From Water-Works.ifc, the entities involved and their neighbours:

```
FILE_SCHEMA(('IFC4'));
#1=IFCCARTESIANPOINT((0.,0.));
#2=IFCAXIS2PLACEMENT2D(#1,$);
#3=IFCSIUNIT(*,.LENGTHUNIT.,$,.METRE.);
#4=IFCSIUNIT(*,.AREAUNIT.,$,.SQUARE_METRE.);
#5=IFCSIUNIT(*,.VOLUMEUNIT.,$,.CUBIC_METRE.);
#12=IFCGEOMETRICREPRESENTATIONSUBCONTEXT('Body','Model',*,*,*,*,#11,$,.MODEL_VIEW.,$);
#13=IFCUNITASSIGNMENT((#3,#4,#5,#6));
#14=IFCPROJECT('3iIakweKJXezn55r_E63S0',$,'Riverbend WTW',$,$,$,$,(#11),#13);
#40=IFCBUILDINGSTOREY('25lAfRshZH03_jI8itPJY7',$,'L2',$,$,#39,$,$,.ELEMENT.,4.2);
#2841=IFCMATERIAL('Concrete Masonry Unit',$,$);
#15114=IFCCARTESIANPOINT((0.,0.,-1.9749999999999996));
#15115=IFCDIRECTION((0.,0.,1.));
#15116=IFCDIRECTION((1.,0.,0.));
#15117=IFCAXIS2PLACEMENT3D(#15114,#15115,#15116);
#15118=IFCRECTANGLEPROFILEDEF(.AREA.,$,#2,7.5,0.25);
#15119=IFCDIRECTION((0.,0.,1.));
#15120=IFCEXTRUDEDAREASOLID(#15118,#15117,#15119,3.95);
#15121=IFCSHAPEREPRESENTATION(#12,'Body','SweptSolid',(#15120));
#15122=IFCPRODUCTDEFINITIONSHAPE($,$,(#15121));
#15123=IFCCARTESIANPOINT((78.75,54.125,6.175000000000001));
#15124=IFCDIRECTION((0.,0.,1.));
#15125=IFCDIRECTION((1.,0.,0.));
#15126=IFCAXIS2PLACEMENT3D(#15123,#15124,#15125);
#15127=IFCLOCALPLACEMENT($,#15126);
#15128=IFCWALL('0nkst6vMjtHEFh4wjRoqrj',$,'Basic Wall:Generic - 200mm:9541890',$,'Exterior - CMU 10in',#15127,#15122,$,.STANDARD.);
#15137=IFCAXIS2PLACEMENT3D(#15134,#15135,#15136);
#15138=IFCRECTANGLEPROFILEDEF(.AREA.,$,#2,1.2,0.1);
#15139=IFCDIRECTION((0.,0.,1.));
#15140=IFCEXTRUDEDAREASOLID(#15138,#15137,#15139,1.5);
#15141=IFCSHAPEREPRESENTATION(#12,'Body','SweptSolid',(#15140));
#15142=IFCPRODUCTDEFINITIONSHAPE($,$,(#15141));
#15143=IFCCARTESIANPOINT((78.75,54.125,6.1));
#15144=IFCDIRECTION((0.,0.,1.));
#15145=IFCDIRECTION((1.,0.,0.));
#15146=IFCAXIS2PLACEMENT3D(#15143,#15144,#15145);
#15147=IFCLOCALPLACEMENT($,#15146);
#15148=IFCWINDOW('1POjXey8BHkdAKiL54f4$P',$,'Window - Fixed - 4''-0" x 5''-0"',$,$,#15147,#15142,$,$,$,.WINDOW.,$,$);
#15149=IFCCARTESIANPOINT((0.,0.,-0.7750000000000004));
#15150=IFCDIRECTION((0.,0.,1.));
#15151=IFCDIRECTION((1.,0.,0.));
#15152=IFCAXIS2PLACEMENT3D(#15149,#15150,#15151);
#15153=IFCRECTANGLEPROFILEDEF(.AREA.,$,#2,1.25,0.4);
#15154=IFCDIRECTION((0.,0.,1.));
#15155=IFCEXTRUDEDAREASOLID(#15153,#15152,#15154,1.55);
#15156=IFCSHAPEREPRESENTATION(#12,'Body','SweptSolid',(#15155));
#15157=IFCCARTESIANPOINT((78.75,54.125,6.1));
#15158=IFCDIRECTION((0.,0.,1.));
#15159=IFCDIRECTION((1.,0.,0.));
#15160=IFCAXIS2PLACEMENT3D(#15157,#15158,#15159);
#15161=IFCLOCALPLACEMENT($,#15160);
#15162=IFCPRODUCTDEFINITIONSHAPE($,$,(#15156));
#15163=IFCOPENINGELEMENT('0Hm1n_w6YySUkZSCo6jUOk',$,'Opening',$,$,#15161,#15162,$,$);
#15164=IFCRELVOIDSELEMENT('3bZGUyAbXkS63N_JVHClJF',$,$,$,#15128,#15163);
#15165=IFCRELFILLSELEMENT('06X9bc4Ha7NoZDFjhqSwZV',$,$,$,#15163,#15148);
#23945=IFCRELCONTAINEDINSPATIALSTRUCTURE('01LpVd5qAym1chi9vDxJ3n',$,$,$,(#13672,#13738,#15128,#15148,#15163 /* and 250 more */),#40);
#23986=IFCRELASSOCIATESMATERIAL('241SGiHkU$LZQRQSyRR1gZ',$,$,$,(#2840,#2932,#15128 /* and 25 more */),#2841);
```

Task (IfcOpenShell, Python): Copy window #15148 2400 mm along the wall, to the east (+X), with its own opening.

```python
import ifcopenshell
import ifcopenshell.api.feature
import ifcopenshell.api.geometry
import ifcopenshell.api.root
import ifcopenshell.geom
import ifcopenshell.util.element
import ifcopenshell.util.placement
import ifcopenshell.util.shape

model = ifcopenshell.open("Water-Works.ifc")
settings = ifcopenshell.geom.settings()


def volume(element):
    """Net volume in cubic metres, openings subtracted."""
    shape = ifcopenshell.geom.create_shape(settings, element)
    return ifcopenshell.util.shape.get_volume(shape.geometry)


window = model.by_guid("1POjXey8BHkdAKiL54f4$P")
opening = window.FillsVoids[0].RelatingOpeningElement
wall = opening.VoidsElements[0].RelatingBuildingElement
before = volume(wall)
shift = ifcopenshell.util.placement.get_local_placement(wall.ObjectPlacement)[:3, 0] * 2.4

# copy_class copies the void relationship, type, container and properties, but no geometry.
new_opening = ifcopenshell.api.root.copy_class(model, product=opening)
new_opening.Representation = ifcopenshell.util.element.copy_deep(
    model, opening.Representation, exclude=["IfcGeometricRepresentationContext", "IfcRepresentationMap"]
)
new_window = ifcopenshell.api.root.copy_class(model, product=window)
new_window.Representation = ifcopenshell.util.element.copy_deep(
    model, window.Representation, exclude=["IfcGeometricRepresentationContext", "IfcRepresentationMap"]
)
ifcopenshell.api.feature.add_filling(model, opening=new_opening, element=new_window)

for old, new in ((opening, new_opening), (window, new_window)):
    matrix = ifcopenshell.util.placement.get_local_placement(old.ObjectPlacement)
    matrix[:3, 3] += shift
    ifcopenshell.api.geometry.edit_object_placement(model, product=new, matrix=matrix, is_si=False)

after = volume(wall)

print(f"wall volume {before:.3f} -> {after:.3f} m3")

model.write("Water-Works-out.ifc")
```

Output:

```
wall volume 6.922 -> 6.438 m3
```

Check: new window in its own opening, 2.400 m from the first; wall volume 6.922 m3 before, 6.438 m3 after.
